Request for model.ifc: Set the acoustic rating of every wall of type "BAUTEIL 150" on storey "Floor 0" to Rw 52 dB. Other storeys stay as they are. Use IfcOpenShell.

First a look at what the model holds.

```python
import ifcopenshell
import ifcopenshell.util.element

model = ifcopenshell.open("model.ifc")
print(model.schema)
storey = next(s for s in model.by_type("IfcBuildingStorey") if s.Name == "Floor 0")
walls = [e for e in ifcopenshell.util.element.get_decomposition(storey) if e.is_a("IfcWall")]
seen = {}
for e in walls:
    element_type = ifcopenshell.util.element.get_type(e)
    key = (element_type.Name if element_type != e and element_type else None, ifcopenshell.util.element.get_pset(e, "Pset_WallCommon", "AcousticRating"))
    seen[key] = seen.get(key, 0) + 1
for (name, value), count in sorted(seen.items(), key=str):
    print(count, "x", name, "|", value)
```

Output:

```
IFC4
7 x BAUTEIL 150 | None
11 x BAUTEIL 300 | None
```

```python
import ifcopenshell
import ifcopenshell.api.pset
import ifcopenshell.util.element

model = ifcopenshell.open("model.ifc")

storey = next(s for s in model.by_type("IfcBuildingStorey") if s.Name == "Floor 0")
walls = [e for e in ifcopenshell.util.element.get_decomposition(storey) if e.is_a("IfcWall")]

count = 0
for e in walls:
    element_type = ifcopenshell.util.element.get_type(e)
    if element_type in (None, e) or element_type.Name != "BAUTEIL 150":
        continue
    # add_pset returns the element's existing set when there is one.
    pset = ifcopenshell.api.pset.add_pset(model, product=e, name="Pset_WallCommon")
    ifcopenshell.api.pset.edit_pset(model, pset=pset, properties={"AcousticRating": "Rw 52 dB"})
    count += 1

print(count, "walls updated")

model.write("model-out.ifc")
```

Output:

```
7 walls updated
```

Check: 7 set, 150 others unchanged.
